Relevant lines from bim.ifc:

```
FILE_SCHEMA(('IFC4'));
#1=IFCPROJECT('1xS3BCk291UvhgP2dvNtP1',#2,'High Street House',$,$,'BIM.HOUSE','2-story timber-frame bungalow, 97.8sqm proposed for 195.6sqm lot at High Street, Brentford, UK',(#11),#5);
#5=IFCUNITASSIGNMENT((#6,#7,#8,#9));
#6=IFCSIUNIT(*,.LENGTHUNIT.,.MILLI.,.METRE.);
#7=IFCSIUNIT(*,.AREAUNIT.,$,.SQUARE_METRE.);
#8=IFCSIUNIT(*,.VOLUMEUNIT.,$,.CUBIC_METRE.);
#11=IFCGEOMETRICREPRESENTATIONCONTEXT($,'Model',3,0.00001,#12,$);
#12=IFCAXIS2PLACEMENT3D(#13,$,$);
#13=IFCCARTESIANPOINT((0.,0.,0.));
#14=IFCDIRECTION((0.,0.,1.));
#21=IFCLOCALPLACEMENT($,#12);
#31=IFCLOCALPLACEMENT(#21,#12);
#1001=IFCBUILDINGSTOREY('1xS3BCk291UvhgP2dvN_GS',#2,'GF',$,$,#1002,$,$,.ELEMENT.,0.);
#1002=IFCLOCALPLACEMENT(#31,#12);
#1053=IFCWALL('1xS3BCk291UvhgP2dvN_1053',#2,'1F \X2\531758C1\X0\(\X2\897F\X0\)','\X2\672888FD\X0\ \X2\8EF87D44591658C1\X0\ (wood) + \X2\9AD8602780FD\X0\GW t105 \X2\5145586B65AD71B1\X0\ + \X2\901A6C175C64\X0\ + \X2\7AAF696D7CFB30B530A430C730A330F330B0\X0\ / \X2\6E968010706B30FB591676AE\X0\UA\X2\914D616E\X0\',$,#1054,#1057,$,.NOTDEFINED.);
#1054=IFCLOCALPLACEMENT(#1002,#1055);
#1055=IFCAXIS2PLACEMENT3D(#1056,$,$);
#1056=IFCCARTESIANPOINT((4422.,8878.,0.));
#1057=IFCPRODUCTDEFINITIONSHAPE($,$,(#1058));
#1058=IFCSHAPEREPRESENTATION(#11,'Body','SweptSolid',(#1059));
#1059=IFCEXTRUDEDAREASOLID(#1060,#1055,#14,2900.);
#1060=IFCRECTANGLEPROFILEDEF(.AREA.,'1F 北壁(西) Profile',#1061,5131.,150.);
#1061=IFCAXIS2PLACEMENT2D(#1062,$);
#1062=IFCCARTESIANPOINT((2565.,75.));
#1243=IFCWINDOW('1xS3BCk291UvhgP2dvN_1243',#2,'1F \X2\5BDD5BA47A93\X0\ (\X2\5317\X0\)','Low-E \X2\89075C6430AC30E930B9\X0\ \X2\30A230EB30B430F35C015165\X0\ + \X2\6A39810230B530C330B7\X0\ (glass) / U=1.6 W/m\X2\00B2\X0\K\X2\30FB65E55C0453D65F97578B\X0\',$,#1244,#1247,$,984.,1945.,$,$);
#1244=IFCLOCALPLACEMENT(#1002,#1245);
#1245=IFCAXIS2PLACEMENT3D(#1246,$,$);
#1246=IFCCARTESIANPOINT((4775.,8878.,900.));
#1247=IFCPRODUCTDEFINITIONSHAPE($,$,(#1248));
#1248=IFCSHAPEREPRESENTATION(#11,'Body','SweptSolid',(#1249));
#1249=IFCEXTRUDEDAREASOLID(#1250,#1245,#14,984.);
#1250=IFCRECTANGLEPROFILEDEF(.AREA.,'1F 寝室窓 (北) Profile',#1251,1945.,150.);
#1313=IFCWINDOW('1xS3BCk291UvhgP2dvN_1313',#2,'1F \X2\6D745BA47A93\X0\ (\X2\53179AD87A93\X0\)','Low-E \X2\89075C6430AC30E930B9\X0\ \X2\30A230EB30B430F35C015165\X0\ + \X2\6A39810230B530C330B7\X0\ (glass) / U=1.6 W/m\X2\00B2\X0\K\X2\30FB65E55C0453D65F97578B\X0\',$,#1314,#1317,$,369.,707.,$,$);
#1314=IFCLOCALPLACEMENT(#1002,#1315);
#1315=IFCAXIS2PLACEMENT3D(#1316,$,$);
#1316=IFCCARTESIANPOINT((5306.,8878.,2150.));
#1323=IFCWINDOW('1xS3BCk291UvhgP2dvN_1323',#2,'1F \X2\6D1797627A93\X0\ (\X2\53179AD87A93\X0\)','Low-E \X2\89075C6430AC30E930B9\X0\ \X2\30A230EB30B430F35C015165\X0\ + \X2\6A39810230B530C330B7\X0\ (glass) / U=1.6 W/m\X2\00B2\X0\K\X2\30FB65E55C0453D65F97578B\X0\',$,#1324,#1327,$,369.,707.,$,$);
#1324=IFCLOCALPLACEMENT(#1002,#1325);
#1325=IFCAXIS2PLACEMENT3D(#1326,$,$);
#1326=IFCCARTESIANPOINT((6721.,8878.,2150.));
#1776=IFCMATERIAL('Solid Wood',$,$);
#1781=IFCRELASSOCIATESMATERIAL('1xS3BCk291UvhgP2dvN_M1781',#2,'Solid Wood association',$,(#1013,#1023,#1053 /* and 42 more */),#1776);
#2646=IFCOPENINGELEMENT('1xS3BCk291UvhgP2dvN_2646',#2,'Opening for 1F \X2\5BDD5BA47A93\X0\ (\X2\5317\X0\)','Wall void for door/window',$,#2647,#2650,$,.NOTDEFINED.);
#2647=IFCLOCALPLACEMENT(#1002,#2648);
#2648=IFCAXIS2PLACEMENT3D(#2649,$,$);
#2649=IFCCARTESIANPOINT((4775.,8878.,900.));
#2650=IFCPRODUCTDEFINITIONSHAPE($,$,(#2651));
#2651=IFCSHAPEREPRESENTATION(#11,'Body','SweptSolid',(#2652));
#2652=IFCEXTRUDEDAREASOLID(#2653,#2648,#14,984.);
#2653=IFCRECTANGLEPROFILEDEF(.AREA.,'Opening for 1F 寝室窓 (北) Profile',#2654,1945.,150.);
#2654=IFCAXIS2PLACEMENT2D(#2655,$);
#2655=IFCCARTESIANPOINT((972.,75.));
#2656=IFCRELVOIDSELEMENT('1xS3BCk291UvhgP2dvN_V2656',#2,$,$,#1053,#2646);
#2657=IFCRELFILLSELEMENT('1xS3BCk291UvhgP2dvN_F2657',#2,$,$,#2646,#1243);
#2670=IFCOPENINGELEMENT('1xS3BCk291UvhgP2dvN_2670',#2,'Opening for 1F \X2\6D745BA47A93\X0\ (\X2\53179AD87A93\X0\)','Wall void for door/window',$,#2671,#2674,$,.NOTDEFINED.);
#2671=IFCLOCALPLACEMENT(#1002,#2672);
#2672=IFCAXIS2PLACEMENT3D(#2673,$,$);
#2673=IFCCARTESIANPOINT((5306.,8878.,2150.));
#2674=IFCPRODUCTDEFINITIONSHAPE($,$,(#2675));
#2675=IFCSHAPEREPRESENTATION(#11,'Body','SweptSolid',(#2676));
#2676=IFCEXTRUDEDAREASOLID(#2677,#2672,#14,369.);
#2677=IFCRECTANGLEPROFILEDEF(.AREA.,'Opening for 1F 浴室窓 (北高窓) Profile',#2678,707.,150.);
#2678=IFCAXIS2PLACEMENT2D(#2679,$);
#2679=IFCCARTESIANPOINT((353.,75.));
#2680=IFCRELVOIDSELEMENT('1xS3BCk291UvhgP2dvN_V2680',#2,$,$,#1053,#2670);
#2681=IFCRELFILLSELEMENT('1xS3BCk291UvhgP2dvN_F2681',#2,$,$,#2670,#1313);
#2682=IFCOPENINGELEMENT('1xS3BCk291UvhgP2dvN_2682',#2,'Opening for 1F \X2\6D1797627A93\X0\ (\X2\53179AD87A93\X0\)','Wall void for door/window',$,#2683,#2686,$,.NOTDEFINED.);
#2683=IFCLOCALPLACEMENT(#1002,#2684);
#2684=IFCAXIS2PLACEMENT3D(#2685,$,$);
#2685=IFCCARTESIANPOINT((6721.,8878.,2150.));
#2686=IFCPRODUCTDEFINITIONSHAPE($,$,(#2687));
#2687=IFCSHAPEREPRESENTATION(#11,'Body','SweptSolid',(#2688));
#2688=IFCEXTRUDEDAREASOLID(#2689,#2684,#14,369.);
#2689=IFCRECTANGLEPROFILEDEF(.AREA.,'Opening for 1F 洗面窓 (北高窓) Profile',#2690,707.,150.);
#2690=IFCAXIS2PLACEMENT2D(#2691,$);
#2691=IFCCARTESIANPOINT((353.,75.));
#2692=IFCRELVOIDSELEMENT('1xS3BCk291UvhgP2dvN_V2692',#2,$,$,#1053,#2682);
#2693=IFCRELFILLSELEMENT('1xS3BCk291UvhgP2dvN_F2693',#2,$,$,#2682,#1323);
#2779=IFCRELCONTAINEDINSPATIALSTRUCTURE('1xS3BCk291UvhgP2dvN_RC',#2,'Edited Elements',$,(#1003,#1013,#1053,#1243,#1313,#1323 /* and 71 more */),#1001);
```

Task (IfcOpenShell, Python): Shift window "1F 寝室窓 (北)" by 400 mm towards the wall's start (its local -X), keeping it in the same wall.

```python
import ifcopenshell
import ifcopenshell.api.geometry
import ifcopenshell.util.placement

model = ifcopenshell.open("bim.ifc")

window = model.by_guid("1xS3BCk291UvhgP2dvN_1243")
opening = window.FillsVoids[0].RelatingOpeningElement
wall = opening.VoidsElements[0].RelatingBuildingElement

wall_matrix = ifcopenshell.util.placement.get_local_placement(wall.ObjectPlacement)
shift = wall_matrix[:3, 0] * -400.0
before = ifcopenshell.util.placement.get_local_placement(window.ObjectPlacement)[:3, 3].copy()

# The window is not placed relative to its opening, so move both.
for product in (opening, window):
    matrix = ifcopenshell.util.placement.get_local_placement(product.ObjectPlacement)
    matrix[:3, 3] += shift
    ifcopenshell.api.geometry.edit_object_placement(model, product=product, matrix=matrix, is_si=False)

after = ifcopenshell.util.placement.get_local_placement(window.ObjectPlacement)[:3, 3]
print("window moved by", (after - before).round(3) + 0.0)

model.write("bim_v2.ifc")
```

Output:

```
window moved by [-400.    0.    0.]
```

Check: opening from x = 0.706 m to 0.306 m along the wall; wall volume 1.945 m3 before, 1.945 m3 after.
